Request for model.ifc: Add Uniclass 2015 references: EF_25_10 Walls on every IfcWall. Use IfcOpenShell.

First a look at what the model holds.

```python
import ifcopenshell

model = ifcopenshell.open("model.ifc")
print(model.schema)
print("classifications:", [c.Name for c in model.by_type("IfcClassification")])
for ifc_class in ("IfcDoor", "IfcRoof", "IfcStair", "IfcWall", "IfcWindow"):
    print(ifc_class, len(model.by_type(ifc_class)))
```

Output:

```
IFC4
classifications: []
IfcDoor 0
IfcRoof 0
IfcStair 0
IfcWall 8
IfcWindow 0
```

```python
import ifcopenshell
import ifcopenshell.api.classification

model = ifcopenshell.open("model.ifc")

system = ifcopenshell.api.classification.add_classification(model, classification="Uniclass 2015")

codes = {
    "IfcWall": ("EF_25_10", "Walls"),
}
for ifc_class, (code, name) in codes.items():
    products = model.by_type(ifc_class)
    ifcopenshell.api.classification.add_reference(
        model, products=products, classification=system, identification=code, name=name
    )
    print(code, len(products))

model.write("model_updated.ifc")
```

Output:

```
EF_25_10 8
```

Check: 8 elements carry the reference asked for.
